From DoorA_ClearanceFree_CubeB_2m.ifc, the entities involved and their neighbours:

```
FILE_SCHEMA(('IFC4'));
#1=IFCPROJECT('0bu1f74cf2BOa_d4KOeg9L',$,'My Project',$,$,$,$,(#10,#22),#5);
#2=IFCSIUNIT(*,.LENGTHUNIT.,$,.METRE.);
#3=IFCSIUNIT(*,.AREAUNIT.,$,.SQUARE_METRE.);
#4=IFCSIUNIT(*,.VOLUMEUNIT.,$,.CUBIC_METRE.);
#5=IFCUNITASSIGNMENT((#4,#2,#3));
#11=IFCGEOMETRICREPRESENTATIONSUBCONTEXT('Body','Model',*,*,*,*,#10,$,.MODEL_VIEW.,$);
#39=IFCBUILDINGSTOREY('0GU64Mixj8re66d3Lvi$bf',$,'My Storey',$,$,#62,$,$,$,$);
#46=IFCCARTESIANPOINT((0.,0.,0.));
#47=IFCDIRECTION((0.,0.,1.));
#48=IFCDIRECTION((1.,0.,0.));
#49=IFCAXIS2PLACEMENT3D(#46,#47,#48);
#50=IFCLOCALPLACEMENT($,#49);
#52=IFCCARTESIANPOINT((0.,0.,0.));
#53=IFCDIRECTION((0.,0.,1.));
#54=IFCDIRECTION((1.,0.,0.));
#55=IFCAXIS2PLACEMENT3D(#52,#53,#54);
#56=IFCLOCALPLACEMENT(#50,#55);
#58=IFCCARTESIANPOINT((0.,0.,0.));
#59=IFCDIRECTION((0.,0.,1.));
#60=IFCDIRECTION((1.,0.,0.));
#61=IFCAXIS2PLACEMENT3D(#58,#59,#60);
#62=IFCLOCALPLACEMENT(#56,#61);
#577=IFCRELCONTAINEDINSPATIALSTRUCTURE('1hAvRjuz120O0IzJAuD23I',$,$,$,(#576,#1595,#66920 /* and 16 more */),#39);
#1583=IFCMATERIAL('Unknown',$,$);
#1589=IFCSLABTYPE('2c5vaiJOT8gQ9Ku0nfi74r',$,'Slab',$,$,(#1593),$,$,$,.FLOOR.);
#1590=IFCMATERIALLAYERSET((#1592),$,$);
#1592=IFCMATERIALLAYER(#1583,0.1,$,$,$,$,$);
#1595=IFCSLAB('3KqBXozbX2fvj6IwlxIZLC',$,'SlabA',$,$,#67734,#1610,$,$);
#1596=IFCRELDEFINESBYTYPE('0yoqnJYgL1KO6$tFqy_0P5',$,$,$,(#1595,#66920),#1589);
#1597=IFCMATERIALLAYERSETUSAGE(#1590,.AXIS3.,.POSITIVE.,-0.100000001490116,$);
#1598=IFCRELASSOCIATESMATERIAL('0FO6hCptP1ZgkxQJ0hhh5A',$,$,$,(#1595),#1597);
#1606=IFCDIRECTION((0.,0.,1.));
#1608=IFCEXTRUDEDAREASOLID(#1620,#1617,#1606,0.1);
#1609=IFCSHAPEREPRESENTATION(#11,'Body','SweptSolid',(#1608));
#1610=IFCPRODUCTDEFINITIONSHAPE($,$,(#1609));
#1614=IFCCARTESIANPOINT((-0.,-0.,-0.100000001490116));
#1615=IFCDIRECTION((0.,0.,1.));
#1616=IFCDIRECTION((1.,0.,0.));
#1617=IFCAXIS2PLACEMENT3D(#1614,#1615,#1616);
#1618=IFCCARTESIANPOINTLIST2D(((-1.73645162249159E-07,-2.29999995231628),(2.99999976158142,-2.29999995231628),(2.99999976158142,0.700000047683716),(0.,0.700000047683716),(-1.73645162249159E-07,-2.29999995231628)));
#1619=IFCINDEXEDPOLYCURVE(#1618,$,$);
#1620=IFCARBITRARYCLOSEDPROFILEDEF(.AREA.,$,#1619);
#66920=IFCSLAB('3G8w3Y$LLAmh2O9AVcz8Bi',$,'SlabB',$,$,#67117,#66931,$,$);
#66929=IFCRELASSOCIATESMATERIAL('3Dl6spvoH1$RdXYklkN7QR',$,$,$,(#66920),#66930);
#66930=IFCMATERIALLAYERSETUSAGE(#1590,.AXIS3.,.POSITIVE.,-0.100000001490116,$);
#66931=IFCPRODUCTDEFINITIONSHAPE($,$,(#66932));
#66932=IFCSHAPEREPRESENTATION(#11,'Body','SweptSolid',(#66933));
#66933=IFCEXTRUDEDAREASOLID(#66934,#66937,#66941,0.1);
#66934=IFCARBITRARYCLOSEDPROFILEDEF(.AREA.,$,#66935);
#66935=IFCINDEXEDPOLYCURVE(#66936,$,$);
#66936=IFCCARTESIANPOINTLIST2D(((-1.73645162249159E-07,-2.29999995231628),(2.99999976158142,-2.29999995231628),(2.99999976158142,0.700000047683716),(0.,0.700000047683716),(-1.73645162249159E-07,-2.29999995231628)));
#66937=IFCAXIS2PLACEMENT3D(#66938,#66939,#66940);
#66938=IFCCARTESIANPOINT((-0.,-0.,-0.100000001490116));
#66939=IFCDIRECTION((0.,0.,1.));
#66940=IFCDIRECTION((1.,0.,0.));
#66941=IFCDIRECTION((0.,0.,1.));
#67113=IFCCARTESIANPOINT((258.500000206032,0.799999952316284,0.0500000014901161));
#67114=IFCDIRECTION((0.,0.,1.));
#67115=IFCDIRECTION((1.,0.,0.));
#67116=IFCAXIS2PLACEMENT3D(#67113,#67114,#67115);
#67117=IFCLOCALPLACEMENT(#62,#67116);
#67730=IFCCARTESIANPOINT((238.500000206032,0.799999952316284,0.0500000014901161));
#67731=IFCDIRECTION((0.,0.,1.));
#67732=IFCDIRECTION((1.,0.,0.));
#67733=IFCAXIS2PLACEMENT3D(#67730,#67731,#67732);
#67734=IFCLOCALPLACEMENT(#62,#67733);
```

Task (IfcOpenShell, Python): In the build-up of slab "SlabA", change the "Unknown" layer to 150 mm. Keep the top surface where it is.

```python
import ifcopenshell
import ifcopenshell.util.element
import ifcopenshell.util.representation

model = ifcopenshell.open("DoorA_ClearanceFree_CubeB_2m.ifc")

layer_set = model.by_id(1590)
layer = next(l for l in layer_set.MaterialLayers if l.Material and l.Material.Name == "Unknown")
change = 0.15 - layer.LayerThickness
layer.LayerThickness += change

# The layer set is shared, so every slab that uses it gets the new thickness.
slabs = [e for e in ifcopenshell.util.element.get_elements_by_material(model, layer_set) if e.is_a("IfcSlab")]
for slab in sorted(slabs, key=lambda e: e.id()):
    body = ifcopenshell.util.representation.get_representation(slab, "Model", "Body")
    solid = body.Items[0]
    old_depth = solid.Depth
    solid.Depth += change
    # Extruded upwards: lower the start of the extrusion so the top stays.
    x, y, z = solid.Position.Location.Coordinates
    solid.Position.Location = model.createIfcCartesianPoint((x, y, z - change))
    print(slab.id(), f"{old_depth:g} -> {solid.Depth:g}")

# The layers are counted up from the underside, which has moved.
for usage in {ifcopenshell.util.element.get_material(slab) for slab in slabs}:
    usage.OffsetFromReferenceLine -= change

model.write("DoorA_ClearanceFree_CubeB_2m_rev.ifc")
```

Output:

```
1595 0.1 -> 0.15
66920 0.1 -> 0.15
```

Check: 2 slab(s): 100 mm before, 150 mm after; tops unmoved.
